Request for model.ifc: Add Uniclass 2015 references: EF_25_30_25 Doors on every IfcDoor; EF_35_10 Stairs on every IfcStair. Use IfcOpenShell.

First a look at what the model holds.

```python
import ifcopenshell

model = ifcopenshell.open("model.ifc")
print(model.schema)
print("classifications:", [c.Name for c in model.by_type("IfcClassification")])
for ifc_class in ("IfcDoor", "IfcRoof", "IfcStair", "IfcWall", "IfcWindow"):
    print(ifc_class, len(model.by_type(ifc_class)))
```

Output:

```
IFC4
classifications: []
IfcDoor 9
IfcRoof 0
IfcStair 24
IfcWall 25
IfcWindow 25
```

```python
import ifcopenshell
import ifcopenshell.api.classification

model = ifcopenshell.open("model.ifc")

system = ifcopenshell.api.classification.add_classification(model, classification="Uniclass 2015")

codes = {
    "IfcDoor": ("EF_25_30_25", "Doors"),
    "IfcStair": ("EF_35_10", "Stairs"),
}
for ifc_class, (code, name) in codes.items():
    products = model.by_type(ifc_class)
    ifcopenshell.api.classification.add_reference(
        model, products=products, classification=system, identification=code, name=name
    )
    print(code, len(products))

model.write("model_rev.ifc")
```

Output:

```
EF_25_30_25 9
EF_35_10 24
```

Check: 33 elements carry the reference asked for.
